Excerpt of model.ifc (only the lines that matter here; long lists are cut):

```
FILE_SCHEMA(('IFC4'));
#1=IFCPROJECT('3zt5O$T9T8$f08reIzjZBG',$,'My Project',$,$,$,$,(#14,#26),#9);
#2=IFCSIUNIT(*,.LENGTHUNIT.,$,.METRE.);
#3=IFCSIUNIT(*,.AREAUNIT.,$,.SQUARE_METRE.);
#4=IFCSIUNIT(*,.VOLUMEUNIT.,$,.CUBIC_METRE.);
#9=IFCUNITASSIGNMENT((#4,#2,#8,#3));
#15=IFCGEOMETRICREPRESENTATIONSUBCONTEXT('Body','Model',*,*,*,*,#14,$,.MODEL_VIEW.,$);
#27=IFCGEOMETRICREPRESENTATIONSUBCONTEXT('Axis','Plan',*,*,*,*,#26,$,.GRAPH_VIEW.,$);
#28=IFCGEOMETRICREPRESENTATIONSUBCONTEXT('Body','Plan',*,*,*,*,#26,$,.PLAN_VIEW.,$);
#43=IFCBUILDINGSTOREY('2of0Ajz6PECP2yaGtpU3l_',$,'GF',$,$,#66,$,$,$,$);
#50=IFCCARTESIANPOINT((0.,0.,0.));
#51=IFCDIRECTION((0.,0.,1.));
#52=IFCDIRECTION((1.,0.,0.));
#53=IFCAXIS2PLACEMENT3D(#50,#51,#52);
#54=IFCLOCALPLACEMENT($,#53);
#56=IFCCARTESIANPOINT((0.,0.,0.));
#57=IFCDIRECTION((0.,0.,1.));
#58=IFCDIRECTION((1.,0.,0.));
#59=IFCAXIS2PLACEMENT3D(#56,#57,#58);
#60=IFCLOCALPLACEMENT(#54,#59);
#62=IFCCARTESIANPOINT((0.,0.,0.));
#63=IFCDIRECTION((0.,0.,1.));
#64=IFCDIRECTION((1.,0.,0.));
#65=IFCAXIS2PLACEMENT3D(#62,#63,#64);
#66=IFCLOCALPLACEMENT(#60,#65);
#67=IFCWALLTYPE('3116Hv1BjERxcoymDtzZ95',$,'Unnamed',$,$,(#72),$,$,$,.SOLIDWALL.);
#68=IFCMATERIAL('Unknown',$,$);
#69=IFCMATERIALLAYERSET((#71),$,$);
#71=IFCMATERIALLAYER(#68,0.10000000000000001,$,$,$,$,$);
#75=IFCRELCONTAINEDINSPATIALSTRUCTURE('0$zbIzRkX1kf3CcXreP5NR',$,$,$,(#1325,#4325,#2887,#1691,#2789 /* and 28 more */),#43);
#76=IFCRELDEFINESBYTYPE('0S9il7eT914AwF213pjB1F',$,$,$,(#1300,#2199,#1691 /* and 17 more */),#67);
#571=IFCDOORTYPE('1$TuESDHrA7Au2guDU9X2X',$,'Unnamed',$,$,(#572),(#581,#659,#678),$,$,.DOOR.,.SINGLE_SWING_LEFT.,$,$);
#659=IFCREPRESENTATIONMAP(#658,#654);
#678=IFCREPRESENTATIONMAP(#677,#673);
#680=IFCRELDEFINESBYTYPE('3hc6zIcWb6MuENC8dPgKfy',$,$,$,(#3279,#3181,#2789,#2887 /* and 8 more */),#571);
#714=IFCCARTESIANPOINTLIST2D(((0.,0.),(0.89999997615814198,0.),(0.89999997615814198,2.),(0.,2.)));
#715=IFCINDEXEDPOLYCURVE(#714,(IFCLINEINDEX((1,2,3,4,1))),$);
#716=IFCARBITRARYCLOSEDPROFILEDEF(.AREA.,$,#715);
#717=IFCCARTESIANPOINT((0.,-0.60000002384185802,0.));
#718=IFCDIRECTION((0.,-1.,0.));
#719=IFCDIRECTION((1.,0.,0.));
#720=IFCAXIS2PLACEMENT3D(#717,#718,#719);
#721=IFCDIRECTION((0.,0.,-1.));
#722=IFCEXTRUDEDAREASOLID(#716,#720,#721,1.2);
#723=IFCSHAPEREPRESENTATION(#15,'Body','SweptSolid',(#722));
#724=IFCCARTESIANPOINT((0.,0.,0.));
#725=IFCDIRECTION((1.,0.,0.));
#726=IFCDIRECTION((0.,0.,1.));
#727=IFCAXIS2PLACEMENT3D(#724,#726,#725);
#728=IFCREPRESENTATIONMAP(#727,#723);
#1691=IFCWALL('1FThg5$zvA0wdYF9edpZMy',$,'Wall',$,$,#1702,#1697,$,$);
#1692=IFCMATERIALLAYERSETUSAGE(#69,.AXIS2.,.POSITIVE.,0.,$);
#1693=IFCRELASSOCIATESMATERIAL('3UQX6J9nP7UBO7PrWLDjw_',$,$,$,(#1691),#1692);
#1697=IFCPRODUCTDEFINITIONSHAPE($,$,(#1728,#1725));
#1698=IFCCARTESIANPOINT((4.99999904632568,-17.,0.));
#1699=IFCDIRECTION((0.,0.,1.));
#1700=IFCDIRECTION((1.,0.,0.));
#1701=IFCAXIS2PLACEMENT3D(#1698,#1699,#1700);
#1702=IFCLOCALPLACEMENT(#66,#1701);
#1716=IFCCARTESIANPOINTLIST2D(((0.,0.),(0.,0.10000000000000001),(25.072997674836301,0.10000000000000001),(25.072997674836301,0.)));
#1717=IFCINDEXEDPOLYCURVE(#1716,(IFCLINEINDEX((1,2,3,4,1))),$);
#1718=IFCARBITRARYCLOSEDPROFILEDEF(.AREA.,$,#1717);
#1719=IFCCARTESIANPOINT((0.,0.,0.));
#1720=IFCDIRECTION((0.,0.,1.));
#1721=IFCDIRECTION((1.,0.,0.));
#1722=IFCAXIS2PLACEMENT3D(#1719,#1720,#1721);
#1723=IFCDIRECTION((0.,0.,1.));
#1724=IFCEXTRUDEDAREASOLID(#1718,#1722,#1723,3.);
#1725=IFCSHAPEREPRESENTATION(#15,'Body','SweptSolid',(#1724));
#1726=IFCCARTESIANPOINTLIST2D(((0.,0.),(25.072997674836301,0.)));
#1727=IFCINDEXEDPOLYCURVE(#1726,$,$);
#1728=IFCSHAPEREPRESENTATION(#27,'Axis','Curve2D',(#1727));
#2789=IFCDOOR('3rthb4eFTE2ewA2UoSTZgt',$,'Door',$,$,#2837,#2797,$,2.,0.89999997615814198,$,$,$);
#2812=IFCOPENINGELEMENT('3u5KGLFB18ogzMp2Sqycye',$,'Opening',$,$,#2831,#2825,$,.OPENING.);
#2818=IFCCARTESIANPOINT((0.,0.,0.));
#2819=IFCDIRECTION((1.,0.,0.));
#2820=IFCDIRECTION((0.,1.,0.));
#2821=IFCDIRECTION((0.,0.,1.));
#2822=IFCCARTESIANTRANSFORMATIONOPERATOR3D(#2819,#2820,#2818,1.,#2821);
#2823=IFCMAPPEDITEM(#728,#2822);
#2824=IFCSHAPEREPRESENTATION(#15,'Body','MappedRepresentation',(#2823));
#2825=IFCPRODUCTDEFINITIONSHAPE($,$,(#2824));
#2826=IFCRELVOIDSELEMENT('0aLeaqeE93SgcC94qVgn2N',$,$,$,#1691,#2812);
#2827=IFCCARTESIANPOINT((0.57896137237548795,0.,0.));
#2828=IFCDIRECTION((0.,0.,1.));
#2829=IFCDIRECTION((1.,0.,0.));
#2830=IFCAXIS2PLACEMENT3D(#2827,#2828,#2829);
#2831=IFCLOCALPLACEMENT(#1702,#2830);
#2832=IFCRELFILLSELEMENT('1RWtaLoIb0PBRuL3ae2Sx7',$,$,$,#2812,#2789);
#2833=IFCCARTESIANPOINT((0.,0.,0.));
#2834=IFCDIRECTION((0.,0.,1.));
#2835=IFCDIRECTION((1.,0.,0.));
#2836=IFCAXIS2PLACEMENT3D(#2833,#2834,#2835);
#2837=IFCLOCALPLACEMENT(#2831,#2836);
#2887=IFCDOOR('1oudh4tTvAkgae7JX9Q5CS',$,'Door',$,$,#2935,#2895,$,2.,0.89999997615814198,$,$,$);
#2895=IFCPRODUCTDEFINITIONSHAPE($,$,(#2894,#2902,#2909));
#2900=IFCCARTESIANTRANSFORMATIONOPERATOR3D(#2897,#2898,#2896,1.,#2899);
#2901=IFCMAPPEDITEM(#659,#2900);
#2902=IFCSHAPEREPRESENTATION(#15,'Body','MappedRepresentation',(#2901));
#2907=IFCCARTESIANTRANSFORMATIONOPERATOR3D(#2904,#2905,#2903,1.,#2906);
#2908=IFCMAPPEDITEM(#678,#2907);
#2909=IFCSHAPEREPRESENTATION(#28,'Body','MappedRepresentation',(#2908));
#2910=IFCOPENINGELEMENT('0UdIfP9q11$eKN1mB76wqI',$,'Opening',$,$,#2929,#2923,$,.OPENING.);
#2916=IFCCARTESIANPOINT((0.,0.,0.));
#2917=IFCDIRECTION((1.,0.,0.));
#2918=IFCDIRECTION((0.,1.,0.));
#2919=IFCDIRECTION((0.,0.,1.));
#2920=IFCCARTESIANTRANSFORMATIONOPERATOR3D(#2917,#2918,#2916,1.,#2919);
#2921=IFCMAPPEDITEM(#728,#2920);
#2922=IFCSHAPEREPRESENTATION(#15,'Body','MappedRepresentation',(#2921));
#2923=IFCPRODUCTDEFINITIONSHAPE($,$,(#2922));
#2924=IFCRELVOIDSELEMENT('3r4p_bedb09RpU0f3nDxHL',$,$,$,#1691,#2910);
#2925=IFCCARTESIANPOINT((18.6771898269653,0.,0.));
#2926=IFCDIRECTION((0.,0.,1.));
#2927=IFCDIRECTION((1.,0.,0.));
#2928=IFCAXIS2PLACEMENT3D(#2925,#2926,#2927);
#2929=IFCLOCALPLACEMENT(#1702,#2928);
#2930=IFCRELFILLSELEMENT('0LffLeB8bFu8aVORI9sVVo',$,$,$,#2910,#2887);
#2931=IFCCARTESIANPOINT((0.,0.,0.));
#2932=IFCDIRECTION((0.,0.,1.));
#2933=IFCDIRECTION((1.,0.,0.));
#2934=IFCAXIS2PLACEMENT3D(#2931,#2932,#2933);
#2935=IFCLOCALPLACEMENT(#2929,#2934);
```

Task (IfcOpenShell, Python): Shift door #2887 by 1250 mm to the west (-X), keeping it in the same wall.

```python
import ifcopenshell
import ifcopenshell.api.geometry
import ifcopenshell.util.placement

model = ifcopenshell.open("model.ifc")

door = model.by_guid("1oudh4tTvAkgae7JX9Q5CS")
opening = door.FillsVoids[0].RelatingOpeningElement
wall = opening.VoidsElements[0].RelatingBuildingElement

wall_matrix = ifcopenshell.util.placement.get_local_placement(wall.ObjectPlacement)
shift = wall_matrix[:3, 0] * -1.25
before = ifcopenshell.util.placement.get_local_placement(door.ObjectPlacement)[:3, 3].copy()

# The door is placed relative to its opening, so it follows when the opening moves.
matrix = ifcopenshell.util.placement.get_local_placement(opening.ObjectPlacement)
matrix[:3, 3] += shift
ifcopenshell.api.geometry.edit_object_placement(
    model, product=opening, matrix=matrix, is_si=False, should_transform_children=True
)

after = ifcopenshell.util.placement.get_local_placement(door.ObjectPlacement)[:3, 3]
print("door moved by", (after - before).round(3) + 0.0)

model.write("model-out.ifc")
```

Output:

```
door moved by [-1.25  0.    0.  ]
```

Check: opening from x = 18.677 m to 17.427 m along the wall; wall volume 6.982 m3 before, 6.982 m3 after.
